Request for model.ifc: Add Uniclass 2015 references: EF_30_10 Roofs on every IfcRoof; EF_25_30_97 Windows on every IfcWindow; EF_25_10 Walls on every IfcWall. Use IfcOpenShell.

First a look at what the model holds.

```python
import ifcopenshell

model = ifcopenshell.open("model.ifc")
print(model.schema)
print("classifications:", [c.Name for c in model.by_type("IfcClassification")])
for ifc_class in ("IfcDoor", "IfcRoof", "IfcStair", "IfcWall", "IfcWindow"):
    print(ifc_class, len(model.by_type(ifc_class)))
```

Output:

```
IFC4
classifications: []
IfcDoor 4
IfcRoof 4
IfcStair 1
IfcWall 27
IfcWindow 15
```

```python
import ifcopenshell
import ifcopenshell.api.classification

model = ifcopenshell.open("model.ifc")

system = ifcopenshell.api.classification.add_classification(model, classification="Uniclass 2015")

codes = {
    "IfcRoof": ("EF_30_10", "Roofs"),
    "IfcWindow": ("EF_25_30_97", "Windows"),
    "IfcWall": ("EF_25_10", "Walls"),
}
for ifc_class, (code, name) in codes.items():
    products = model.by_type(ifc_class)
    ifcopenshell.api.classification.add_reference(
        model, products=products, classification=system, identification=code, name=name
    )
    print(code, len(products))

model.write("model_updated.ifc")
```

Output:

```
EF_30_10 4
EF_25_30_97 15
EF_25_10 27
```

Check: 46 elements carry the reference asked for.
